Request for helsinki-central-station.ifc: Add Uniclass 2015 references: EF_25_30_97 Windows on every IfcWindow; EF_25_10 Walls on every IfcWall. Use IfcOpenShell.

First a look at what the model holds.

```python
import ifcopenshell

model = ifcopenshell.open("helsinki-central-station.ifc")
print(model.schema)
print("classifications:", [c.Name for c in model.by_type("IfcClassification")])
for ifc_class in ("IfcDoor", "IfcRoof", "IfcStair", "IfcWall", "IfcWindow"):
    print(ifc_class, len(model.by_type(ifc_class)))
```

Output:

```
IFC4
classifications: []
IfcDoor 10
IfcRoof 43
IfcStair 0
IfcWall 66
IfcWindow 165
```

```python
import ifcopenshell
import ifcopenshell.api.classification

model = ifcopenshell.open("helsinki-central-station.ifc")

system = ifcopenshell.api.classification.add_classification(model, classification="Uniclass 2015")

codes = {
    "IfcWindow": ("EF_25_30_97", "Windows"),
    "IfcWall": ("EF_25_10", "Walls"),
}
for ifc_class, (code, name) in codes.items():
    products = model.by_type(ifc_class)
    ifcopenshell.api.classification.add_reference(
        model, products=products, classification=system, identification=code, name=name
    )
    print(code, len(products))

model.write("helsinki-central-station-out.ifc")
```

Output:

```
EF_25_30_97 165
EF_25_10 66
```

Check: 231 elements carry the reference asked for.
